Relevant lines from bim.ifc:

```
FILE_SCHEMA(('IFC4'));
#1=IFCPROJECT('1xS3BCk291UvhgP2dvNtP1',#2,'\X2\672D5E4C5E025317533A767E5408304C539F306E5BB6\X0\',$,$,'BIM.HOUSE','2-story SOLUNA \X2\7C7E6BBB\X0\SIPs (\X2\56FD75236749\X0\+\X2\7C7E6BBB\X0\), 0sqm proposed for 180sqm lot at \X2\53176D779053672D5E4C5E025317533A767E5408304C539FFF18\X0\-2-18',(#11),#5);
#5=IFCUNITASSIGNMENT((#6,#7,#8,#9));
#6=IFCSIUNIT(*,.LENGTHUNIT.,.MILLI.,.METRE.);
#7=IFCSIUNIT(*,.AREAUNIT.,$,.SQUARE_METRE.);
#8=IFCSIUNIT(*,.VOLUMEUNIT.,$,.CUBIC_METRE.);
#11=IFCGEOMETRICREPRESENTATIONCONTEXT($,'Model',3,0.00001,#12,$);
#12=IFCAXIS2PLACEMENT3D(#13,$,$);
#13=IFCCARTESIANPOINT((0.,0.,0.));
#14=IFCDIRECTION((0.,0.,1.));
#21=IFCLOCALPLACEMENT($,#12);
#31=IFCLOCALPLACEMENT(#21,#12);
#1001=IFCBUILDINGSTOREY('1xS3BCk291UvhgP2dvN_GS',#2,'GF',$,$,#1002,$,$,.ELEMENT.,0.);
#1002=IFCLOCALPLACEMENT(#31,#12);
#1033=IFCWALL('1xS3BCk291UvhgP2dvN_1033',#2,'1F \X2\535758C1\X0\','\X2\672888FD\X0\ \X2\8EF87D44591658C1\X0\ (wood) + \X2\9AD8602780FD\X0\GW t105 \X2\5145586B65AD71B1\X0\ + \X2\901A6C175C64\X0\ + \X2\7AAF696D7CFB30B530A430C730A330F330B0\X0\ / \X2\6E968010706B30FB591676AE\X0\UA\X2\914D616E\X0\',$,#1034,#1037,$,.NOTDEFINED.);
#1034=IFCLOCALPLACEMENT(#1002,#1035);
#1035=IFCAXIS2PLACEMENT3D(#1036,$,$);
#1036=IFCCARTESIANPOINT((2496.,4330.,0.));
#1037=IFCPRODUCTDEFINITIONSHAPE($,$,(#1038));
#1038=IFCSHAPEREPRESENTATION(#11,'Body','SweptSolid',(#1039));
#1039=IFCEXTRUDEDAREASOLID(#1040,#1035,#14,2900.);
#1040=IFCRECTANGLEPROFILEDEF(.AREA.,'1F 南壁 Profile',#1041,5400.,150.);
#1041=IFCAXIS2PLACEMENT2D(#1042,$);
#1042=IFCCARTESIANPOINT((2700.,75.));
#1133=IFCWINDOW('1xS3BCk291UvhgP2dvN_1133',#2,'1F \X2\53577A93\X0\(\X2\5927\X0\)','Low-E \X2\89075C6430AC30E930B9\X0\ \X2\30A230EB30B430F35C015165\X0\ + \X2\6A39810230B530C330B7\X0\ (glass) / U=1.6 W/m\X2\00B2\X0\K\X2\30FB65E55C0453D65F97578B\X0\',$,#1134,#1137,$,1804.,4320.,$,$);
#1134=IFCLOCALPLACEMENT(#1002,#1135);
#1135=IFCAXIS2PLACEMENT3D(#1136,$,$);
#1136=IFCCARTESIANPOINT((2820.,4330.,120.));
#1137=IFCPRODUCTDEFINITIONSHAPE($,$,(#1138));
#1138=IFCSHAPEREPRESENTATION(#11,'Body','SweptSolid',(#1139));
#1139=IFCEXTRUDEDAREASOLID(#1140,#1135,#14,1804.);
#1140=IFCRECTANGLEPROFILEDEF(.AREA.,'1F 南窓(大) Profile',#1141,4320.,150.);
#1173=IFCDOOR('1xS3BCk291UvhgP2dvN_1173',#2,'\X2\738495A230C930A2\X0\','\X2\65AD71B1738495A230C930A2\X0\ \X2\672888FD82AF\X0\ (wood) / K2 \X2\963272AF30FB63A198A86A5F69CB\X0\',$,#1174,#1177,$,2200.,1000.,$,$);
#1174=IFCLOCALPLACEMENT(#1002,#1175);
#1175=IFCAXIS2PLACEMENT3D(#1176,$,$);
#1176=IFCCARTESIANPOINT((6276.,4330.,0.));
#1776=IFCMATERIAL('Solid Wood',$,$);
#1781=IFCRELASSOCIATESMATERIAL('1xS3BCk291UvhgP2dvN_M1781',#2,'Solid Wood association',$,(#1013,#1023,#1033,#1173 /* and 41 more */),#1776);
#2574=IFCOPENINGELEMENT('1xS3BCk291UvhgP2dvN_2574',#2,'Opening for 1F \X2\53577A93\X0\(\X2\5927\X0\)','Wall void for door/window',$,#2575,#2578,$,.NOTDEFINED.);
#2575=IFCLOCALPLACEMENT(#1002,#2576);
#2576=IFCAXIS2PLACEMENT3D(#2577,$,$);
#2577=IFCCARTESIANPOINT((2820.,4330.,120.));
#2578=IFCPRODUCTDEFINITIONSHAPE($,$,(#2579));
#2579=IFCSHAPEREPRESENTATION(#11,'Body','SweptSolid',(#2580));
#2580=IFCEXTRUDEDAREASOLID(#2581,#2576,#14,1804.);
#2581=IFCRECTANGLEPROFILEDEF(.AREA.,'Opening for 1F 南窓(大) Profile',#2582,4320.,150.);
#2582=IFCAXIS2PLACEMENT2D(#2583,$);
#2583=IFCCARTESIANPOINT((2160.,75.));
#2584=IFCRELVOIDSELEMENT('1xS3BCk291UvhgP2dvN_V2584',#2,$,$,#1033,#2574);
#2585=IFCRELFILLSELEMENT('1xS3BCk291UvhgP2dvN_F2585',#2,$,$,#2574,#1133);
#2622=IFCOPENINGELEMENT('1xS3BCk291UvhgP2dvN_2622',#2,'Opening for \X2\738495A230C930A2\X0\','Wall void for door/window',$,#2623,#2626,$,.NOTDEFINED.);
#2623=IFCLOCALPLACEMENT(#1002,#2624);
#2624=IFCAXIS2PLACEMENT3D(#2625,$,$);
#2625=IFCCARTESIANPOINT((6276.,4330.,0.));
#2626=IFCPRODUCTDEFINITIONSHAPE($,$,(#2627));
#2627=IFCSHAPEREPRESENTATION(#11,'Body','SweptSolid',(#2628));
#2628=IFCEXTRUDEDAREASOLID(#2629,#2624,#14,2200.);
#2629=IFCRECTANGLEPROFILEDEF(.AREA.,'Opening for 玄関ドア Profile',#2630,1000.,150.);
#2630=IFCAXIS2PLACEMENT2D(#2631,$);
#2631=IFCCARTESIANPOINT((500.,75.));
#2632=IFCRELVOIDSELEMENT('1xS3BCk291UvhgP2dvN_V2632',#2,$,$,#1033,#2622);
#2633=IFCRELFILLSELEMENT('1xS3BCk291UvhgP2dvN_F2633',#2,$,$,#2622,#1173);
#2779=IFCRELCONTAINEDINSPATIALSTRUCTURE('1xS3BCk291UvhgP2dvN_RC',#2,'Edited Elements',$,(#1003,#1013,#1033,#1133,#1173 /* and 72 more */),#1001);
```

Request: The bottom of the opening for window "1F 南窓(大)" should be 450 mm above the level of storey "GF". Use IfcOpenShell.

```python
import numpy as np
import ifcopenshell
import ifcopenshell.api.geometry
import ifcopenshell.geom
import ifcopenshell.util.element
import ifcopenshell.util.placement
import ifcopenshell.util.shape
import ifcopenshell.util.unit

model = ifcopenshell.open("bim.ifc")
unit_scale = ifcopenshell.util.unit.calculate_unit_scale(model)

window = model.by_guid("1xS3BCk291UvhgP2dvN_1133")
opening = window.FillsVoids[0].RelatingOpeningElement
storey = ifcopenshell.util.element.get_container(window, ifc_class="IfcBuildingStorey")
level = ifcopenshell.util.placement.get_local_placement(storey.ObjectPlacement)[2, 3]

# The opening's origin need not be at the sill, so measure its lowest point.
shape = ifcopenshell.geom.create_shape(ifcopenshell.geom.settings(), opening)
bottom = ifcopenshell.util.shape.get_shape_bottom_elevation(shape, shape.geometry) / unit_scale
dz = level + 450.0 - bottom

shift = np.array([0.0, 0.0, dz])
# The window is not placed relative to its opening, so move both.
for product in (opening, window):
    matrix = ifcopenshell.util.placement.get_local_placement(product.ObjectPlacement)
    matrix[:3, 3] += shift
    ifcopenshell.api.geometry.edit_object_placement(model, product=product, matrix=matrix, is_si=False)

print(f"moved by {dz * unit_scale:+.3f} m")

model.write("bim-out.ifc")
```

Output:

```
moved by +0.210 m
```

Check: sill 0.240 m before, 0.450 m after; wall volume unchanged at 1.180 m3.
